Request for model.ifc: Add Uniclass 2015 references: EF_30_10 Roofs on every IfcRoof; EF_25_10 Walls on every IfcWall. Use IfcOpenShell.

First a look at what the model holds.

```python
import ifcopenshell

model = ifcopenshell.open("model.ifc")
print(model.schema)
print("classifications:", [c.Name for c in model.by_type("IfcClassification")])
for ifc_class in ("IfcDoor", "IfcRoof", "IfcStair", "IfcWall", "IfcWindow"):
    print(ifc_class, len(model.by_type(ifc_class)))
```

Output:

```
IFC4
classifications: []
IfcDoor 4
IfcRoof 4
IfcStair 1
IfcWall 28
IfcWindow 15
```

```python
import ifcopenshell
import ifcopenshell.api.classification

model = ifcopenshell.open("model.ifc")

system = ifcopenshell.api.classification.add_classification(model, classification="Uniclass 2015")

codes = {
    "IfcRoof": ("EF_30_10", "Roofs"),
    "IfcWall": ("EF_25_10", "Walls"),
}
for ifc_class, (code, name) in codes.items():
    products = model.by_type(ifc_class)
    ifcopenshell.api.classification.add_reference(
        model, products=products, classification=system, identification=code, name=name
    )
    print(code, len(products))

model.write("model-out.ifc")
```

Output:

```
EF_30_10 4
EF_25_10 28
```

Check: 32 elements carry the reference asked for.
